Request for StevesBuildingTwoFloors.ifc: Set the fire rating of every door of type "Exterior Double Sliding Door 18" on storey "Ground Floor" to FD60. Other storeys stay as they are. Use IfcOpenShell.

First a look at what the model holds.

```python
import ifcopenshell
import ifcopenshell.util.element

model = ifcopenshell.open("StevesBuildingTwoFloors.ifc")
print(model.schema)
storey = next(s for s in model.by_type("IfcBuildingStorey") if s.Name == "Ground Floor")
doors = [e for e in ifcopenshell.util.element.get_decomposition(storey) if e.is_a("IfcDoor")]
seen = {}
for e in doors:
    element_type = ifcopenshell.util.element.get_type(e)
    key = (element_type.Name if element_type != e and element_type else None, ifcopenshell.util.element.get_pset(e, "Pset_DoorCommon", "FireRating"))
    seen[key] = seen.get(key, 0) + 1
for (name, value), count in sorted(seen.items(), key=str):
    print(count, "x", name, "|", value)
```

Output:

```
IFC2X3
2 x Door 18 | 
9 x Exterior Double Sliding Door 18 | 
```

```python
import ifcopenshell
import ifcopenshell.api.pset
import ifcopenshell.util.element

model = ifcopenshell.open("StevesBuildingTwoFloors.ifc")

storey = next(s for s in model.by_type("IfcBuildingStorey") if s.Name == "Ground Floor")
doors = [e for e in ifcopenshell.util.element.get_decomposition(storey) if e.is_a("IfcDoor")]

count = 0
for e in doors:
    element_type = ifcopenshell.util.element.get_type(e)
    if element_type in (None, e) or element_type.Name != "Exterior Double Sliding Door 18":
        continue
    # add_pset returns the element's existing set when there is one.
    pset = ifcopenshell.api.pset.add_pset(model, product=e, name="Pset_DoorCommon")
    ifcopenshell.api.pset.edit_pset(model, pset=pset, properties={"FireRating": "FD60"})
    count += 1

print(count, "doors updated")

model.write("StevesBuildingTwoFloors_edited.ifc")
```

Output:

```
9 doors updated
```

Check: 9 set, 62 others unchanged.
